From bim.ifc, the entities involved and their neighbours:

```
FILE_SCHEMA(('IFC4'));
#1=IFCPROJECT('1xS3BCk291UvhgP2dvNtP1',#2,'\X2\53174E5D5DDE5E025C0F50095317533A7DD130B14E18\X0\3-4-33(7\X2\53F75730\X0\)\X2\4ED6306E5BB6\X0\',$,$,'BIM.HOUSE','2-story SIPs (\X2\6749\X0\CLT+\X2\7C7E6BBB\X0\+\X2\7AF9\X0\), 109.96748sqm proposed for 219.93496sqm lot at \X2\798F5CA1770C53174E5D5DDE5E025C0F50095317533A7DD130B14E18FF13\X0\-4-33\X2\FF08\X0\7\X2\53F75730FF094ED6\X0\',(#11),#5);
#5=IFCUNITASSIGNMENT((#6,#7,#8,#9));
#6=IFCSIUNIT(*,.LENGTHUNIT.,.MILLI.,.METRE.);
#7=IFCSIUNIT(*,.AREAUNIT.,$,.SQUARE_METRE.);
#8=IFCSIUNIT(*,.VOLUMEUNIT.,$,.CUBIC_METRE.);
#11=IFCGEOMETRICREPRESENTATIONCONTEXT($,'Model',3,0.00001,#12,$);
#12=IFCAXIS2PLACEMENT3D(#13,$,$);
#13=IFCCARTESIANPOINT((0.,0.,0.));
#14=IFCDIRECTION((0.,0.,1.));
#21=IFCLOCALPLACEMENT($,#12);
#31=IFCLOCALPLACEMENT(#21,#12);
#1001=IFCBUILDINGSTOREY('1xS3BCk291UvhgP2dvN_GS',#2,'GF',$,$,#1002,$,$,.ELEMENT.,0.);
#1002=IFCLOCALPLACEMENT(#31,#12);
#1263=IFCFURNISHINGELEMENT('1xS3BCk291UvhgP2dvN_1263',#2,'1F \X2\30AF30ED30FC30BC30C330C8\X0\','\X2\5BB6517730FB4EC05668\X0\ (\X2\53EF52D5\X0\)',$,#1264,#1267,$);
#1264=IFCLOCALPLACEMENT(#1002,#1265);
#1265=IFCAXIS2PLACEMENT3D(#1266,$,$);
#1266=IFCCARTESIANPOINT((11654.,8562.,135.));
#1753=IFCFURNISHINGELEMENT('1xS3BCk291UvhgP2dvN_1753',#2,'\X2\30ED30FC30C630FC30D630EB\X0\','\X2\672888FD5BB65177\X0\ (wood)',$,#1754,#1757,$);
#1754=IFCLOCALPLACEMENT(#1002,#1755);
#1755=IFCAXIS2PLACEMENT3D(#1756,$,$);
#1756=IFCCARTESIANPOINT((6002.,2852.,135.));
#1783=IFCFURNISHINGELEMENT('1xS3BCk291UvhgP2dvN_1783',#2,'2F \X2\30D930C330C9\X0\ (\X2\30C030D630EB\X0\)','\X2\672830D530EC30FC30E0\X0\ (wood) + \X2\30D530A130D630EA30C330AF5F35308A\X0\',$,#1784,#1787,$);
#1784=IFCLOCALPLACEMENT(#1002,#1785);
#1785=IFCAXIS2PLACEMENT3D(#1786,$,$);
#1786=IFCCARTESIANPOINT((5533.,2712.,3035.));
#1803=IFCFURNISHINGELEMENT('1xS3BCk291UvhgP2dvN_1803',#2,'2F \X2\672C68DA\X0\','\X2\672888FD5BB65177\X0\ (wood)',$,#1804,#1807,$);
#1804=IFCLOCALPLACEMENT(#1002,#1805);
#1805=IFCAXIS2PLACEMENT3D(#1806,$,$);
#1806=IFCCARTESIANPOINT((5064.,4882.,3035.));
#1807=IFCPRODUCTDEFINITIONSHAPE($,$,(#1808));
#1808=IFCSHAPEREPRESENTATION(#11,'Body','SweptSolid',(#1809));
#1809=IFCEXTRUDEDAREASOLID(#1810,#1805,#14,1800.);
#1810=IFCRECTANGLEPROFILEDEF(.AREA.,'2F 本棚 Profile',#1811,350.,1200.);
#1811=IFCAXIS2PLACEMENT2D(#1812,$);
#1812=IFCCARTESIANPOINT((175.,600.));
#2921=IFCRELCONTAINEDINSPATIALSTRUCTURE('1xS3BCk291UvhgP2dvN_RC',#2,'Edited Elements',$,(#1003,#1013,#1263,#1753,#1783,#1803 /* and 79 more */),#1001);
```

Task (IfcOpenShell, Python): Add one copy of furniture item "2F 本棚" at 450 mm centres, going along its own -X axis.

```python
import ifcopenshell
import ifcopenshell.api.geometry
import ifcopenshell.api.root
import ifcopenshell.util.element
import ifcopenshell.util.placement

model = ifcopenshell.open("bim.ifc")


def reuse_history(source, copy):
    """copy_class also copies each property set's owner history, people and application; keep the originals."""
    for rel in copy.IsDefinedBy:
        if rel.is_a("IfcRelDefinesByProperties") and (history := rel.RelatingPropertyDefinition.OwnerHistory):
            rel.RelatingPropertyDefinition.OwnerHistory = source.OwnerHistory
            ifcopenshell.util.element.remove_deep2(model, history)


source = model.by_guid("1xS3BCk291UvhgP2dvN_1803")
base = ifcopenshell.util.placement.get_local_placement(source.ObjectPlacement)
step = -base[:3, 0] * 450.0

for i in range(1, 2):
    copy = ifcopenshell.api.root.copy_class(model, product=source)
    copy.Representation = ifcopenshell.util.element.copy_deep(
        model, source.Representation, exclude=["IfcGeometricRepresentationContext", "IfcRepresentationMap"]
    )
    reuse_history(source, copy)
    matrix = base.copy()
    matrix[:3, 3] += i * step
    print("added at", matrix[:3, 3].round(3) + 0.0)
    ifcopenshell.api.geometry.edit_object_placement(model, product=copy, matrix=matrix, is_si=False)

model.write("bim_v2.ifc")
```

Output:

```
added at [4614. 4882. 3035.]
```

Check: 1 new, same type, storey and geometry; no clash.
